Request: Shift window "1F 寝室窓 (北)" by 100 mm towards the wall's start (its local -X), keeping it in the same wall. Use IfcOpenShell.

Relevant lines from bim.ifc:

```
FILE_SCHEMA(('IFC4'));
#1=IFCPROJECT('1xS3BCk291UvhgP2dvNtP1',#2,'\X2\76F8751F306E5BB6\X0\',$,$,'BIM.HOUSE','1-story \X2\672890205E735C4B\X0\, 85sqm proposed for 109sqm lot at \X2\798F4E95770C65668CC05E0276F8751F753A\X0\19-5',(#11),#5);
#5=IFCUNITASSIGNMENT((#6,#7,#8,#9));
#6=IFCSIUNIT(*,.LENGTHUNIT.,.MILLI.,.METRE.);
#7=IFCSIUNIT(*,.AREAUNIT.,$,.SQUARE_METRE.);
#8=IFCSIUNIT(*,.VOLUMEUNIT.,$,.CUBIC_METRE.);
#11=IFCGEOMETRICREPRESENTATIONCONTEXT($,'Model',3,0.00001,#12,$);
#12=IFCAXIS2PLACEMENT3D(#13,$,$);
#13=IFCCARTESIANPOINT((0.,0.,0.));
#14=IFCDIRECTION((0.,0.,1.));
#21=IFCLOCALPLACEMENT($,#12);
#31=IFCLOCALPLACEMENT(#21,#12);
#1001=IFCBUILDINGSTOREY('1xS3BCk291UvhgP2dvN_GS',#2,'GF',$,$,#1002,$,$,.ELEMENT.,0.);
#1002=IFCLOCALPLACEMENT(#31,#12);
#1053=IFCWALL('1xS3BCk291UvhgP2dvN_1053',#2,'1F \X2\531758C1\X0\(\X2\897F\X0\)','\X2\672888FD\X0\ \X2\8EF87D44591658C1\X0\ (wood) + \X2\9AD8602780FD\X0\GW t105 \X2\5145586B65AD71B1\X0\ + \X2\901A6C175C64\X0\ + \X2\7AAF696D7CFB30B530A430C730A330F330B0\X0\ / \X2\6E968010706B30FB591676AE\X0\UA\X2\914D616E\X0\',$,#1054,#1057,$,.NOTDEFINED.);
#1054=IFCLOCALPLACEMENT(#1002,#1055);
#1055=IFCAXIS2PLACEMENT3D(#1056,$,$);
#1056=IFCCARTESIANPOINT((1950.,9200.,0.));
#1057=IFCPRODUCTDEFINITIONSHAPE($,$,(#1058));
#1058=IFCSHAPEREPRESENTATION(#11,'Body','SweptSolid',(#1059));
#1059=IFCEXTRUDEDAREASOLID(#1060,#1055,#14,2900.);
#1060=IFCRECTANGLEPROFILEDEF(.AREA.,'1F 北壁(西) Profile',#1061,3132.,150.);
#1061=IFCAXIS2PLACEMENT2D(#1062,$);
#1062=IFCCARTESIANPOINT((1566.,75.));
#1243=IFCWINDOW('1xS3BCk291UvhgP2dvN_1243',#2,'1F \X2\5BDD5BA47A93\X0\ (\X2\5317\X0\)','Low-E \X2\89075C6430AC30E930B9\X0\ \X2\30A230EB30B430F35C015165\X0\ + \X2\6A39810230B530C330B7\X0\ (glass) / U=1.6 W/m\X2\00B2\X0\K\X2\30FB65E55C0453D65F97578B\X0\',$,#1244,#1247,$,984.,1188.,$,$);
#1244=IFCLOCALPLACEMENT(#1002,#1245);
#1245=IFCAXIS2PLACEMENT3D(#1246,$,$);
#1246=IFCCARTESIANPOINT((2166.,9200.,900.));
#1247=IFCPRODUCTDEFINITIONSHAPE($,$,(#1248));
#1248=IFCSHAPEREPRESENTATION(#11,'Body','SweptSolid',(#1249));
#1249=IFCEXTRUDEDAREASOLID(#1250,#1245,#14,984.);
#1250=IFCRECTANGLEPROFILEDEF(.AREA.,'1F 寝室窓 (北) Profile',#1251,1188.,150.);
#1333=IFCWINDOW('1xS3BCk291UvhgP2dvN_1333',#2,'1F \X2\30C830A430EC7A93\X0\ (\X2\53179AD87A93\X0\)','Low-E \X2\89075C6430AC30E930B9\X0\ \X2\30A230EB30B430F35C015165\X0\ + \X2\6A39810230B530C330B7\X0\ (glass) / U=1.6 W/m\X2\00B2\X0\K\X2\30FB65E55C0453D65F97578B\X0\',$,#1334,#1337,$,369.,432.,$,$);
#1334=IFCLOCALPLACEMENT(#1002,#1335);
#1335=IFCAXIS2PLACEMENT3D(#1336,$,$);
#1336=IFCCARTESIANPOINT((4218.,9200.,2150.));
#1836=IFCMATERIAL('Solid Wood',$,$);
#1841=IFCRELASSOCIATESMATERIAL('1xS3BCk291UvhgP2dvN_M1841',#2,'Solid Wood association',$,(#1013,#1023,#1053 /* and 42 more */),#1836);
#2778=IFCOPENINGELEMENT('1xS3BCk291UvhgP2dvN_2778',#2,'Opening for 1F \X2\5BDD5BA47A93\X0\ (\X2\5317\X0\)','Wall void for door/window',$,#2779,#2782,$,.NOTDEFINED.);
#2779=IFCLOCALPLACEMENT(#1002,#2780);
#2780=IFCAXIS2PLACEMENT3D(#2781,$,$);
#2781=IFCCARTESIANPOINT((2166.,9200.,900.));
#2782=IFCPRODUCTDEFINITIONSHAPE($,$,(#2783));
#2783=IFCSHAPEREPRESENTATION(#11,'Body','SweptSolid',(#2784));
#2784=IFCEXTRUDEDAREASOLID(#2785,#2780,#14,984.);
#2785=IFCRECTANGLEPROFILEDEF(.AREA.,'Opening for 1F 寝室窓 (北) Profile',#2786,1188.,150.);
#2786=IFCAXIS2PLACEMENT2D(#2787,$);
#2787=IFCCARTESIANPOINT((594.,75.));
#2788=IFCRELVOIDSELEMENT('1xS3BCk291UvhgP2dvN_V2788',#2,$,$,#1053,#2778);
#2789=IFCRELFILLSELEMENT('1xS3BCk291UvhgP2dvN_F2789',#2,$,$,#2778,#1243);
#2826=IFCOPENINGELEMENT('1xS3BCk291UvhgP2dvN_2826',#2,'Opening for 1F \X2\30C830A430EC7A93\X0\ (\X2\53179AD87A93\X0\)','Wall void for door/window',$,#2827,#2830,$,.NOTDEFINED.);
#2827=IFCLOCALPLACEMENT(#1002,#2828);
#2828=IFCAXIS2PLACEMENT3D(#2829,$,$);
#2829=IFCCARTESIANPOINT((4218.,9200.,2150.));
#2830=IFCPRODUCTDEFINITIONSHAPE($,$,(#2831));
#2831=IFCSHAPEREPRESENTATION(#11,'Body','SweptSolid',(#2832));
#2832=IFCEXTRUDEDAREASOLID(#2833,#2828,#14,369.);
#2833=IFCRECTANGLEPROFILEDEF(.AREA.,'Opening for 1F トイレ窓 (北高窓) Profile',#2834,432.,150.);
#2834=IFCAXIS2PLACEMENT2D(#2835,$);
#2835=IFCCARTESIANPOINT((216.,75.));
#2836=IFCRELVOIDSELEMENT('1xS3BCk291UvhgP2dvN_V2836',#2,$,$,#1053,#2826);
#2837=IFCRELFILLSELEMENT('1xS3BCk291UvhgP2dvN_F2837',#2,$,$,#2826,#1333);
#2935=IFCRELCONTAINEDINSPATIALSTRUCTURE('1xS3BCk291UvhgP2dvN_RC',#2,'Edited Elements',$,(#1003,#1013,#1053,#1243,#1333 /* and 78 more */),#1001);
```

```python
import ifcopenshell
import ifcopenshell.api.geometry
import ifcopenshell.util.placement

model = ifcopenshell.open("bim.ifc")

window = model.by_guid("1xS3BCk291UvhgP2dvN_1243")
opening = window.FillsVoids[0].RelatingOpeningElement
wall = opening.VoidsElements[0].RelatingBuildingElement

wall_matrix = ifcopenshell.util.placement.get_local_placement(wall.ObjectPlacement)
shift = wall_matrix[:3, 0] * -100.0
before = ifcopenshell.util.placement.get_local_placement(window.ObjectPlacement)[:3, 3].copy()

# The window is not placed relative to its opening, so move both.
for product in (opening, window):
    matrix = ifcopenshell.util.placement.get_local_placement(product.ObjectPlacement)
    matrix[:3, 3] += shift
    ifcopenshell.api.geometry.edit_object_placement(model, product=product, matrix=matrix, is_si=False)

after = ifcopenshell.util.placement.get_local_placement(window.ObjectPlacement)[:3, 3]
print("window moved by", (after - before).round(3) + 0.0)

model.write("bim-out.ifc")
```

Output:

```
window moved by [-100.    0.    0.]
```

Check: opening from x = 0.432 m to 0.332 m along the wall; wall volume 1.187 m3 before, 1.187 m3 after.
